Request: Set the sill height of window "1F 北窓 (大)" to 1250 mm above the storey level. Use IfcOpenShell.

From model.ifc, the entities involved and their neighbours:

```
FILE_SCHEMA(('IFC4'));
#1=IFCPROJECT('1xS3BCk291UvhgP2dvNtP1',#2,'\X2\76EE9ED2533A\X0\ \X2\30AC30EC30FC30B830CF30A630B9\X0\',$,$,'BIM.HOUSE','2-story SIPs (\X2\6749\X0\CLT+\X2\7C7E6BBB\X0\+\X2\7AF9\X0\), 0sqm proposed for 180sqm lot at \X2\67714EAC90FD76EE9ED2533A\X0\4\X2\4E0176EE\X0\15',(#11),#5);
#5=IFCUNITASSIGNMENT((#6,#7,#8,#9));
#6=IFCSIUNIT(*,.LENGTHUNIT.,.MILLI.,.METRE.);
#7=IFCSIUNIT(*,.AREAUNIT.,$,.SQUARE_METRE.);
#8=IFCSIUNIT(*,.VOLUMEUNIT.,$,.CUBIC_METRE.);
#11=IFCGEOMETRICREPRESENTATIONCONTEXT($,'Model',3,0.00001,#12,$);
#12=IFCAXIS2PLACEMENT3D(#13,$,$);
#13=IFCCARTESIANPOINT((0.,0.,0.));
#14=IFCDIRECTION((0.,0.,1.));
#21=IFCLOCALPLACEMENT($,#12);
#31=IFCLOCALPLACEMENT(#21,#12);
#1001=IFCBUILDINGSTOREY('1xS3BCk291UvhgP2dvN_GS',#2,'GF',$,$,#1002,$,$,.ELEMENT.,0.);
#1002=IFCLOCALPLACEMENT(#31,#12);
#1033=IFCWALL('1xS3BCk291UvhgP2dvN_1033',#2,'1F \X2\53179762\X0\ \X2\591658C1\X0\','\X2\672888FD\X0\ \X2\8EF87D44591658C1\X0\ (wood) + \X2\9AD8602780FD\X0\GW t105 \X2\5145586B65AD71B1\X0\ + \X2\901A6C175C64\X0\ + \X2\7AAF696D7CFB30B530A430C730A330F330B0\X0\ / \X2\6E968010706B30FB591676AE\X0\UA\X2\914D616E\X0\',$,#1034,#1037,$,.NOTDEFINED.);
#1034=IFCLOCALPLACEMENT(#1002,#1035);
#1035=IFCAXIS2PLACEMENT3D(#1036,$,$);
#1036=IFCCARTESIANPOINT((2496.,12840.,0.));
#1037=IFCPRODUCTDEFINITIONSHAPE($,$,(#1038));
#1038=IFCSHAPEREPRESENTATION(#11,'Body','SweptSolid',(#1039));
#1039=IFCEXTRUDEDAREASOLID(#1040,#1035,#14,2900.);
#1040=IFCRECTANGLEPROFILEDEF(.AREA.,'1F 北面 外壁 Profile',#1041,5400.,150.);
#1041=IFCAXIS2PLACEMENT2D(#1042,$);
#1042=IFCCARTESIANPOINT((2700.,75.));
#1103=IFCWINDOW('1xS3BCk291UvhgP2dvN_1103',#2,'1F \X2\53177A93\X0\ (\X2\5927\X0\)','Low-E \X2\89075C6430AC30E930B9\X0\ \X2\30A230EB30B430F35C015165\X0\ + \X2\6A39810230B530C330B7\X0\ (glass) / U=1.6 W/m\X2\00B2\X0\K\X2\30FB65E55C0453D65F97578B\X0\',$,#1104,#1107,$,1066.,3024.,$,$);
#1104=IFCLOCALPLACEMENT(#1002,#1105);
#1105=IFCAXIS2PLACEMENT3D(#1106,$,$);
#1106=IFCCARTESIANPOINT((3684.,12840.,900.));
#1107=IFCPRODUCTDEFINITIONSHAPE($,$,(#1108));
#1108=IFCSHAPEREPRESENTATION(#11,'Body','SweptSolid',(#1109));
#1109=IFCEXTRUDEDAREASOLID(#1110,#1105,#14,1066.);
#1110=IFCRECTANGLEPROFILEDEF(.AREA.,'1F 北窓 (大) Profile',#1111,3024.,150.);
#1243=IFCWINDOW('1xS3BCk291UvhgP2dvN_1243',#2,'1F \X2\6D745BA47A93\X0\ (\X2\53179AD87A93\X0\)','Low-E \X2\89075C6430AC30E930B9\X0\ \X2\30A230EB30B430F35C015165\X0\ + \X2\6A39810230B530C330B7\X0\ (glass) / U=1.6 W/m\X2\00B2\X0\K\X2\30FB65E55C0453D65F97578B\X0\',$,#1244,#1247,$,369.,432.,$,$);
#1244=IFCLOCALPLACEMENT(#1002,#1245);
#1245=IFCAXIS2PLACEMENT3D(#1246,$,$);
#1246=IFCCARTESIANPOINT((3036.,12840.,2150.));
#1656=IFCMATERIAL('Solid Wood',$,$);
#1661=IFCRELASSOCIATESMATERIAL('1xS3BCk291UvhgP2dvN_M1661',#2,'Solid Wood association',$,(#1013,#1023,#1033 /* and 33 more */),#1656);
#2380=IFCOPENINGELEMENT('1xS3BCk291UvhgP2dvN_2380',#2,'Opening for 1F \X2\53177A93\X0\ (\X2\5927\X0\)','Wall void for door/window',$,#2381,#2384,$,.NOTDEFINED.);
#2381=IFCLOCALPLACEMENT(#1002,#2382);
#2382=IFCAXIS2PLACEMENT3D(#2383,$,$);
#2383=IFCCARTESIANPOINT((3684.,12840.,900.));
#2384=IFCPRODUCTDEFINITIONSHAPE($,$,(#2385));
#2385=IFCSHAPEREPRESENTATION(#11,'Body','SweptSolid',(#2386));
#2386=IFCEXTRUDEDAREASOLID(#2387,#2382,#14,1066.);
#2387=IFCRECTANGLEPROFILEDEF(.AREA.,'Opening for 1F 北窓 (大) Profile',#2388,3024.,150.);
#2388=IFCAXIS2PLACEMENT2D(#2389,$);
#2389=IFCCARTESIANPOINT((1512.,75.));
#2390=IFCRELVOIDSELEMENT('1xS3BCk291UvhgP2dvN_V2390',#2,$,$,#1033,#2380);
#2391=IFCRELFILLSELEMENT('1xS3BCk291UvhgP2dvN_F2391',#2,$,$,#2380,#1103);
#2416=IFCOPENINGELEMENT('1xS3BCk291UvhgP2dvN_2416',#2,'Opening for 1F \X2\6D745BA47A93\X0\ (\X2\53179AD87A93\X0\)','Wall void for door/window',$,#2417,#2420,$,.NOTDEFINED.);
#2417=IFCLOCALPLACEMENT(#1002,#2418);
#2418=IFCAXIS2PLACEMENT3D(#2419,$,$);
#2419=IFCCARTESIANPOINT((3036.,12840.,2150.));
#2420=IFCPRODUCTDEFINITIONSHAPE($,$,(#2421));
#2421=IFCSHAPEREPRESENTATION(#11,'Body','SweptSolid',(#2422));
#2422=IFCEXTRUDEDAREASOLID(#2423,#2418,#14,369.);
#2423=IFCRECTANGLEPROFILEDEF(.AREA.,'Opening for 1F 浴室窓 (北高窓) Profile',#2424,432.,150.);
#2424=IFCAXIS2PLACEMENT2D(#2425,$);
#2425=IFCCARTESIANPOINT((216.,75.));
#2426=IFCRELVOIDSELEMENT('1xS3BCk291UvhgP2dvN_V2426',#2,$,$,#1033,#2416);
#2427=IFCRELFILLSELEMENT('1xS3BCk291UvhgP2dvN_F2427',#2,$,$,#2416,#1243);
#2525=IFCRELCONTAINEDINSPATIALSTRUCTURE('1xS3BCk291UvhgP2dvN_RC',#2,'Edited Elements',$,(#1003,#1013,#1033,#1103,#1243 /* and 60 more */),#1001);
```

```python
import numpy as np
import ifcopenshell
import ifcopenshell.api.geometry
import ifcopenshell.geom
import ifcopenshell.util.element
import ifcopenshell.util.placement
import ifcopenshell.util.shape
import ifcopenshell.util.unit

model = ifcopenshell.open("model.ifc")
unit_scale = ifcopenshell.util.unit.calculate_unit_scale(model)

window = model.by_guid("1xS3BCk291UvhgP2dvN_1103")
opening = window.FillsVoids[0].RelatingOpeningElement
storey = ifcopenshell.util.element.get_container(window, ifc_class="IfcBuildingStorey")
level = ifcopenshell.util.placement.get_local_placement(storey.ObjectPlacement)[2, 3]

# The opening's origin need not be at the sill, so measure its lowest point.
shape = ifcopenshell.geom.create_shape(ifcopenshell.geom.settings(), opening)
bottom = ifcopenshell.util.shape.get_shape_bottom_elevation(shape, shape.geometry) / unit_scale
dz = level + 1250.0 - bottom

shift = np.array([0.0, 0.0, dz])
# The window is not placed relative to its opening, so move both.
for product in (opening, window):
    matrix = ifcopenshell.util.placement.get_local_placement(product.ObjectPlacement)
    matrix[:3, 3] += shift
    ifcopenshell.api.geometry.edit_object_placement(model, product=product, matrix=matrix, is_si=False)

print(f"moved by {dz * unit_scale:+.3f} m")

model.write("model_updated.ifc")
```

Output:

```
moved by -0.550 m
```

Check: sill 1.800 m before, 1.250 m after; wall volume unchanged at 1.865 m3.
